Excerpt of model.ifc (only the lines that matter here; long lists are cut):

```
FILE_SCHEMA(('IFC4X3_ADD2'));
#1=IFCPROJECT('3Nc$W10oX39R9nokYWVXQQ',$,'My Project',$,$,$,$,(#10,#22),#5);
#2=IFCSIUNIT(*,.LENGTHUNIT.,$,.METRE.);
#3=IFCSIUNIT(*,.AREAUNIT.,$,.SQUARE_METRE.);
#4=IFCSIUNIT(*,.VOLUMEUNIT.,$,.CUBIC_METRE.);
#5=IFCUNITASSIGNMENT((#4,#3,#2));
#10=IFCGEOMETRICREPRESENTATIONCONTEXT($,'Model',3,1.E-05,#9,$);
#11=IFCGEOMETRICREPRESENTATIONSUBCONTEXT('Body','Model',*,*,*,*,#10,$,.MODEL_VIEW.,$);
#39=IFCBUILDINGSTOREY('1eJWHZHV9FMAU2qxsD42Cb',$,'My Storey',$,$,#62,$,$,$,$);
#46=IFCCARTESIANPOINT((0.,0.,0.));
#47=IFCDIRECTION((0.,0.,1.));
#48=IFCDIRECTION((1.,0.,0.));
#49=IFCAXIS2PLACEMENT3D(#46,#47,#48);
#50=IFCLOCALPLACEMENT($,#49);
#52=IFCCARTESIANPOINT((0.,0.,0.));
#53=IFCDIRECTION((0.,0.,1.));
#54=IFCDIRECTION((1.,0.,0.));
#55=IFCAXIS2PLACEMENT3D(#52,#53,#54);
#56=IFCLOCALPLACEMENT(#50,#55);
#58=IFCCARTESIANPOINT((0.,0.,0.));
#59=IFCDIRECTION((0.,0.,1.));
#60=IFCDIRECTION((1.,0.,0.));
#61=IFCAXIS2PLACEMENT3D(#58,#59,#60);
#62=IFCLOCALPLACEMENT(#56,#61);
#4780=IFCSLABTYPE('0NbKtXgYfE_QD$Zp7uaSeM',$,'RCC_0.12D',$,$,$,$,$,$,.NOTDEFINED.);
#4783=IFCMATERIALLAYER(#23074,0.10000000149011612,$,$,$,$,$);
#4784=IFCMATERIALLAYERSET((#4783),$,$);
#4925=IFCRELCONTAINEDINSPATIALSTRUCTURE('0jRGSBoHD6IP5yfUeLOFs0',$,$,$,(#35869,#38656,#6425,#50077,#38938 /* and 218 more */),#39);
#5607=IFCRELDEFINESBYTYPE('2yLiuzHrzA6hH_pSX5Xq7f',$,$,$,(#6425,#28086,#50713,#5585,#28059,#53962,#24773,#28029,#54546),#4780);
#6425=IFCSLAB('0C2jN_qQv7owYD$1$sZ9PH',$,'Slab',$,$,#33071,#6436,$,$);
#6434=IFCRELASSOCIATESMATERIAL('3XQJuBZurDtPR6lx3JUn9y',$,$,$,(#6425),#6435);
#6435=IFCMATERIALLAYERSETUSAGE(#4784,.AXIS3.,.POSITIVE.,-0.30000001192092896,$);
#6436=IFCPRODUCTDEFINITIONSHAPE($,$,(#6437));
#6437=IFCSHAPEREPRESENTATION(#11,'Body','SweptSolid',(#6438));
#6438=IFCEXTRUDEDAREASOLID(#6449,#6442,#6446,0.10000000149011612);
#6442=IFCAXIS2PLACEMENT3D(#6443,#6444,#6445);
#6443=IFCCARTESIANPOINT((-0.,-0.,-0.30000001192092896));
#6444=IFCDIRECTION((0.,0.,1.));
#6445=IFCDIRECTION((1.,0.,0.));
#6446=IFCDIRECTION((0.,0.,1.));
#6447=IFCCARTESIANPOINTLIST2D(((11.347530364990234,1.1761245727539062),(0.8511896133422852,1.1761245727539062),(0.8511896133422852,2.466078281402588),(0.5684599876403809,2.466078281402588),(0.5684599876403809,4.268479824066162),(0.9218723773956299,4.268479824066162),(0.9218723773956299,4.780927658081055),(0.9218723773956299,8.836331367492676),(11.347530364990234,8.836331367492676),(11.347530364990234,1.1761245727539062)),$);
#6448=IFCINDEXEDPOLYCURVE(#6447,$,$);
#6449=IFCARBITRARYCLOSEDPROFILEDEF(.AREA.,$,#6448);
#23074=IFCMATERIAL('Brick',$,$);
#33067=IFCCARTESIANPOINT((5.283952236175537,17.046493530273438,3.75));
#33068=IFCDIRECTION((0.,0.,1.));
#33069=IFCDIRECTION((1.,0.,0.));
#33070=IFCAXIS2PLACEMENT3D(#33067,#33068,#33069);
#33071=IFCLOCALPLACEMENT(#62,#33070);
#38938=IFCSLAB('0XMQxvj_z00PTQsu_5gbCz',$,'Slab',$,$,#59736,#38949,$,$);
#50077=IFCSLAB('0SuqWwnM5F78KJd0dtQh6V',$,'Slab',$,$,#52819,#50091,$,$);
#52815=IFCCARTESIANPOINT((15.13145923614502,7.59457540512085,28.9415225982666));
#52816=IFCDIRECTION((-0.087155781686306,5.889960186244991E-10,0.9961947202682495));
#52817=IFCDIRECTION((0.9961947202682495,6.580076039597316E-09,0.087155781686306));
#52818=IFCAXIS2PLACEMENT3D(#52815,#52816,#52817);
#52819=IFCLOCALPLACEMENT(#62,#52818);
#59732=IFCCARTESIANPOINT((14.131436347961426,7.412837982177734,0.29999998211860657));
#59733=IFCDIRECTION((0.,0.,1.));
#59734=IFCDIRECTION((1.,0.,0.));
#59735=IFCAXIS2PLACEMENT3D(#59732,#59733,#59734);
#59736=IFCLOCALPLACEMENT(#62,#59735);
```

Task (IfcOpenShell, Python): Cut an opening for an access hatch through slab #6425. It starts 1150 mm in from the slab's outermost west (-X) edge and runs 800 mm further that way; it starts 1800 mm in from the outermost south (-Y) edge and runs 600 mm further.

```python
import numpy as np
import ifcopenshell
import ifcopenshell.api.feature
import ifcopenshell.api.geometry
import ifcopenshell.api.root
import ifcopenshell.geom
import ifcopenshell.util.placement
import ifcopenshell.util.representation
import ifcopenshell.util.shape
import ifcopenshell.util.unit

model = ifcopenshell.open("model.ifc")
unit_scale = ifcopenshell.util.unit.calculate_unit_scale(model)
settings = ifcopenshell.geom.settings()


def volume(element):
    """Net volume in cubic metres, openings subtracted."""
    shape = ifcopenshell.geom.create_shape(settings, element)
    return ifcopenshell.util.shape.get_volume(shape.geometry)


slab = model.by_id(6425)
before = volume(slab)

# Extent in the slab's own axes, in metres. The edges named are its -X and -Y sides.
slab_shape = ifcopenshell.geom.create_shape(settings, slab)
vertices = ifcopenshell.util.shape.get_vertices(slab_shape.geometry)
x_min, y_min, bottom = vertices.min(axis=0)
top = vertices[:, 2].max()

opening = ifcopenshell.api.root.create_entity(model, ifc_class="IfcOpeningElement", name="Access hatch opening", predefined_type="OPENING")
context = ifcopenshell.util.representation.get_context(model, "Model", "Body", "MODEL_VIEW")
width, depth = 0.8, 0.6
outline = [(0.0, 0.0), (width, 0.0), (width, depth), (0.0, depth), (0.0, 0.0)]
# Overshoot both faces by 50 mm so the cut is clean.
shape = ifcopenshell.api.geometry.add_slab_representation(
    model, context=context, depth=top - bottom + 0.1, polyline=outline
)
ifcopenshell.api.geometry.assign_representation(model, product=opening, representation=shape)

matrix = ifcopenshell.util.placement.get_local_placement(slab.ObjectPlacement)
matrix[:, 3] = matrix @ np.append(np.array([x_min + 1.15, y_min + 1.8, bottom - 0.05]) / unit_scale, 1.0)
ifcopenshell.api.geometry.edit_object_placement(model, product=opening, matrix=matrix, is_si=False)
ifcopenshell.api.feature.add_feature(model, feature=opening, element=slab)

after = volume(slab)

print(f"slab volume {before:.3f} -> {after:.3f} m3")

model.write("model_rev.ifc")
```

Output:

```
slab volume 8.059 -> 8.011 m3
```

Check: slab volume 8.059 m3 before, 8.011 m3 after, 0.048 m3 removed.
